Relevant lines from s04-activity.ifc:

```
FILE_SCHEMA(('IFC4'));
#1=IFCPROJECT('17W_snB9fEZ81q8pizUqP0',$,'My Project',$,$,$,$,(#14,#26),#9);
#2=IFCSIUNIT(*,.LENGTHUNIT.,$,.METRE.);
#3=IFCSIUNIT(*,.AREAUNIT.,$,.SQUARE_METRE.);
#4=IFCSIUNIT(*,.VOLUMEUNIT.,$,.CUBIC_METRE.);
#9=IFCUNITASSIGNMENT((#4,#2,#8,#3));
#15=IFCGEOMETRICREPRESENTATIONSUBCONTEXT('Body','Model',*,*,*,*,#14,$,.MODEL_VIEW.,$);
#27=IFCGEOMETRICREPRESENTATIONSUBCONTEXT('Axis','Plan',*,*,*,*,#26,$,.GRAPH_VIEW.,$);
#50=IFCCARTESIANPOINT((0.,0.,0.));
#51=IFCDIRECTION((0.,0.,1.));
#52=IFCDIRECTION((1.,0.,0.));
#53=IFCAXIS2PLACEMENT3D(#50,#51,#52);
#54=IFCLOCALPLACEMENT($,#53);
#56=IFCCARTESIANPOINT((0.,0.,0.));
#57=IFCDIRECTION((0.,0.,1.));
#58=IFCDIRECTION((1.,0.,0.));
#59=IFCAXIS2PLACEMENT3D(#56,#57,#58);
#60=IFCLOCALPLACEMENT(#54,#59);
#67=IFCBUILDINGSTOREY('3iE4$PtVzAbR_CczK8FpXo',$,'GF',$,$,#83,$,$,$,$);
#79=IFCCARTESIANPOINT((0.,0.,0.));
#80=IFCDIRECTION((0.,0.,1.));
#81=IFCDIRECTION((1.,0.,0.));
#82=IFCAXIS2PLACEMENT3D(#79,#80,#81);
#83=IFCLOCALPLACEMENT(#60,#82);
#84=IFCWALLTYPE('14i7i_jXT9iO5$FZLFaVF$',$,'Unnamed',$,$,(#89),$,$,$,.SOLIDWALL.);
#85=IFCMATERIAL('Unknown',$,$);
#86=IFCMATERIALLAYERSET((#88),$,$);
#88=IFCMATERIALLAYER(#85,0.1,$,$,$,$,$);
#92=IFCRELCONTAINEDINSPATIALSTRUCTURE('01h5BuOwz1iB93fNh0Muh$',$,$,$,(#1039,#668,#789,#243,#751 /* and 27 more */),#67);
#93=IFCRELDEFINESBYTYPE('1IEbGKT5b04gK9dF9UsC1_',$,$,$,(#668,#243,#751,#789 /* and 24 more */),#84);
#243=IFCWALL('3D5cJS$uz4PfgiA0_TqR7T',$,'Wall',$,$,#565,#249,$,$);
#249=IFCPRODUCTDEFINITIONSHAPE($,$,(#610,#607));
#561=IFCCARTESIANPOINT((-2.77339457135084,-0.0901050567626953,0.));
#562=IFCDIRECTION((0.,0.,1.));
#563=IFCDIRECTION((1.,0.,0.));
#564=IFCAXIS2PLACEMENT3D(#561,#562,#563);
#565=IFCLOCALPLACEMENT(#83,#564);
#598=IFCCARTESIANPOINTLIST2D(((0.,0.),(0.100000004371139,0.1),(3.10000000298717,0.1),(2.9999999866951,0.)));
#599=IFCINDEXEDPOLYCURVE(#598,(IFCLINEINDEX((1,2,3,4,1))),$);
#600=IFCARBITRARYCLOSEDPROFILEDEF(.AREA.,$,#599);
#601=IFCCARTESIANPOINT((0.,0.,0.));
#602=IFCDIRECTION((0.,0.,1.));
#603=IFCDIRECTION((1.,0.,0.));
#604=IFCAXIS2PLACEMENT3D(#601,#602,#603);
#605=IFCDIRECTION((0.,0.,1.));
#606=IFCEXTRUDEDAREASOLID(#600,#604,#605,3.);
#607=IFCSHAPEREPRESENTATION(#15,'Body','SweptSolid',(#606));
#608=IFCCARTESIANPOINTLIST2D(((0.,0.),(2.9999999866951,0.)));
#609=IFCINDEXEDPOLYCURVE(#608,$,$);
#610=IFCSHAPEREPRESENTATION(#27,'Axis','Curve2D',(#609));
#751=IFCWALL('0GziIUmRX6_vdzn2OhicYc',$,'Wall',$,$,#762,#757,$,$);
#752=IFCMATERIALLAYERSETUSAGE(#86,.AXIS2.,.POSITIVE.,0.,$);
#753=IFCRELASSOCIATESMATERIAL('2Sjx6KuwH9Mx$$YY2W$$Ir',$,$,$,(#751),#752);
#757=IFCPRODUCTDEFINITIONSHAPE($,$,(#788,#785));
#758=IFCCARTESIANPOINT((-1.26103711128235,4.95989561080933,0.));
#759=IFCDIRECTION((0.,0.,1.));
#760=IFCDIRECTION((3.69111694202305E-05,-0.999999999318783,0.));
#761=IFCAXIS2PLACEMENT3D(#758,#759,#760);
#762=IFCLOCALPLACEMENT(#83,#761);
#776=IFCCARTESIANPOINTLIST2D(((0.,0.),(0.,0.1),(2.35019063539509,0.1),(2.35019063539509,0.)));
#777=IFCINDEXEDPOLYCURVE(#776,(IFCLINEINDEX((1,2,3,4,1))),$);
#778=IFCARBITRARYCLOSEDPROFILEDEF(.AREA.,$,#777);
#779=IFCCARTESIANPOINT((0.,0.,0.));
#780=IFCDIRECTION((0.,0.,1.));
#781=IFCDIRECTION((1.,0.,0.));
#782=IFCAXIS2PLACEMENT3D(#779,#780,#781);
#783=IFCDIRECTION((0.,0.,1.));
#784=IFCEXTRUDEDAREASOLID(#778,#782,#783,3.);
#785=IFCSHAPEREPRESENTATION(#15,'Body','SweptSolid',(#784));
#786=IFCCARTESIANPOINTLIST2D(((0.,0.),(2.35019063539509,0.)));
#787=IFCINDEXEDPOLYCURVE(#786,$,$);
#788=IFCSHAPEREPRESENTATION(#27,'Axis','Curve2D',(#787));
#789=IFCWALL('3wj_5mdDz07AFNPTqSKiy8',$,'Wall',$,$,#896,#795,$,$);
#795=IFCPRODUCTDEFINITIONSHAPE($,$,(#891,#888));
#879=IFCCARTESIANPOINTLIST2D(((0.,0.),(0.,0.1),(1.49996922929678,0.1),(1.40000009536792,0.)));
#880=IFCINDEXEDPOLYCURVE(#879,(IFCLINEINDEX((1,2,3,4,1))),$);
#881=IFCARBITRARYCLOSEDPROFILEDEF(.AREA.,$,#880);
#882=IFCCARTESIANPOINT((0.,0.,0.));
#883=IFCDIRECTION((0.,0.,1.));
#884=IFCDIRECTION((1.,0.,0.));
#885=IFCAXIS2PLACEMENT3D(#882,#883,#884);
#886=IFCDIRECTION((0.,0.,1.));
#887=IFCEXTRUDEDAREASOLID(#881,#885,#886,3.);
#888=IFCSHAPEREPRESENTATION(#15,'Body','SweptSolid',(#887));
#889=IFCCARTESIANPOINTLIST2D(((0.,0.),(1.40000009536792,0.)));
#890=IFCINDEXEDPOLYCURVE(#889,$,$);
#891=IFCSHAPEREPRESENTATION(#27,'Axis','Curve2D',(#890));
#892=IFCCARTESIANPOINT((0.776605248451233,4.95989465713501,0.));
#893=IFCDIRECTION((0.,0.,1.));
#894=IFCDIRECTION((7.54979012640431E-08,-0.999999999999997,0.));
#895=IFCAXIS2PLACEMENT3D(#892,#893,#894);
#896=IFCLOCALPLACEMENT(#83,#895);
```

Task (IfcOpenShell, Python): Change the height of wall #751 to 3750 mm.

```python
import ifcopenshell
import ifcopenshell.geom
import ifcopenshell.util.representation
import ifcopenshell.util.shape

model = ifcopenshell.open("s04-activity.ifc")
settings = ifcopenshell.geom.settings()


def volume(element):
    """Net volume in cubic metres, openings subtracted."""
    shape = ifcopenshell.geom.create_shape(settings, element)
    return ifcopenshell.util.shape.get_volume(shape.geometry)


wall = model.by_guid("0GziIUmRX6_vdzn2OhicYc")
before = volume(wall)

body = ifcopenshell.util.representation.get_representation(wall, "Model", "Body")
solid = body.Items[0]
old_height = solid.Depth
solid.Depth = 3.75
after = volume(wall)

print(f"height {old_height:g} -> {solid.Depth:g}, volume {before:.3f} -> {after:.3f} m3")

model.write("s04-activity_edited.ifc")
```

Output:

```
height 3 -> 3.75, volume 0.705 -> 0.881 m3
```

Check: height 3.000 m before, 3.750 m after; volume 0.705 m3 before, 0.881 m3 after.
